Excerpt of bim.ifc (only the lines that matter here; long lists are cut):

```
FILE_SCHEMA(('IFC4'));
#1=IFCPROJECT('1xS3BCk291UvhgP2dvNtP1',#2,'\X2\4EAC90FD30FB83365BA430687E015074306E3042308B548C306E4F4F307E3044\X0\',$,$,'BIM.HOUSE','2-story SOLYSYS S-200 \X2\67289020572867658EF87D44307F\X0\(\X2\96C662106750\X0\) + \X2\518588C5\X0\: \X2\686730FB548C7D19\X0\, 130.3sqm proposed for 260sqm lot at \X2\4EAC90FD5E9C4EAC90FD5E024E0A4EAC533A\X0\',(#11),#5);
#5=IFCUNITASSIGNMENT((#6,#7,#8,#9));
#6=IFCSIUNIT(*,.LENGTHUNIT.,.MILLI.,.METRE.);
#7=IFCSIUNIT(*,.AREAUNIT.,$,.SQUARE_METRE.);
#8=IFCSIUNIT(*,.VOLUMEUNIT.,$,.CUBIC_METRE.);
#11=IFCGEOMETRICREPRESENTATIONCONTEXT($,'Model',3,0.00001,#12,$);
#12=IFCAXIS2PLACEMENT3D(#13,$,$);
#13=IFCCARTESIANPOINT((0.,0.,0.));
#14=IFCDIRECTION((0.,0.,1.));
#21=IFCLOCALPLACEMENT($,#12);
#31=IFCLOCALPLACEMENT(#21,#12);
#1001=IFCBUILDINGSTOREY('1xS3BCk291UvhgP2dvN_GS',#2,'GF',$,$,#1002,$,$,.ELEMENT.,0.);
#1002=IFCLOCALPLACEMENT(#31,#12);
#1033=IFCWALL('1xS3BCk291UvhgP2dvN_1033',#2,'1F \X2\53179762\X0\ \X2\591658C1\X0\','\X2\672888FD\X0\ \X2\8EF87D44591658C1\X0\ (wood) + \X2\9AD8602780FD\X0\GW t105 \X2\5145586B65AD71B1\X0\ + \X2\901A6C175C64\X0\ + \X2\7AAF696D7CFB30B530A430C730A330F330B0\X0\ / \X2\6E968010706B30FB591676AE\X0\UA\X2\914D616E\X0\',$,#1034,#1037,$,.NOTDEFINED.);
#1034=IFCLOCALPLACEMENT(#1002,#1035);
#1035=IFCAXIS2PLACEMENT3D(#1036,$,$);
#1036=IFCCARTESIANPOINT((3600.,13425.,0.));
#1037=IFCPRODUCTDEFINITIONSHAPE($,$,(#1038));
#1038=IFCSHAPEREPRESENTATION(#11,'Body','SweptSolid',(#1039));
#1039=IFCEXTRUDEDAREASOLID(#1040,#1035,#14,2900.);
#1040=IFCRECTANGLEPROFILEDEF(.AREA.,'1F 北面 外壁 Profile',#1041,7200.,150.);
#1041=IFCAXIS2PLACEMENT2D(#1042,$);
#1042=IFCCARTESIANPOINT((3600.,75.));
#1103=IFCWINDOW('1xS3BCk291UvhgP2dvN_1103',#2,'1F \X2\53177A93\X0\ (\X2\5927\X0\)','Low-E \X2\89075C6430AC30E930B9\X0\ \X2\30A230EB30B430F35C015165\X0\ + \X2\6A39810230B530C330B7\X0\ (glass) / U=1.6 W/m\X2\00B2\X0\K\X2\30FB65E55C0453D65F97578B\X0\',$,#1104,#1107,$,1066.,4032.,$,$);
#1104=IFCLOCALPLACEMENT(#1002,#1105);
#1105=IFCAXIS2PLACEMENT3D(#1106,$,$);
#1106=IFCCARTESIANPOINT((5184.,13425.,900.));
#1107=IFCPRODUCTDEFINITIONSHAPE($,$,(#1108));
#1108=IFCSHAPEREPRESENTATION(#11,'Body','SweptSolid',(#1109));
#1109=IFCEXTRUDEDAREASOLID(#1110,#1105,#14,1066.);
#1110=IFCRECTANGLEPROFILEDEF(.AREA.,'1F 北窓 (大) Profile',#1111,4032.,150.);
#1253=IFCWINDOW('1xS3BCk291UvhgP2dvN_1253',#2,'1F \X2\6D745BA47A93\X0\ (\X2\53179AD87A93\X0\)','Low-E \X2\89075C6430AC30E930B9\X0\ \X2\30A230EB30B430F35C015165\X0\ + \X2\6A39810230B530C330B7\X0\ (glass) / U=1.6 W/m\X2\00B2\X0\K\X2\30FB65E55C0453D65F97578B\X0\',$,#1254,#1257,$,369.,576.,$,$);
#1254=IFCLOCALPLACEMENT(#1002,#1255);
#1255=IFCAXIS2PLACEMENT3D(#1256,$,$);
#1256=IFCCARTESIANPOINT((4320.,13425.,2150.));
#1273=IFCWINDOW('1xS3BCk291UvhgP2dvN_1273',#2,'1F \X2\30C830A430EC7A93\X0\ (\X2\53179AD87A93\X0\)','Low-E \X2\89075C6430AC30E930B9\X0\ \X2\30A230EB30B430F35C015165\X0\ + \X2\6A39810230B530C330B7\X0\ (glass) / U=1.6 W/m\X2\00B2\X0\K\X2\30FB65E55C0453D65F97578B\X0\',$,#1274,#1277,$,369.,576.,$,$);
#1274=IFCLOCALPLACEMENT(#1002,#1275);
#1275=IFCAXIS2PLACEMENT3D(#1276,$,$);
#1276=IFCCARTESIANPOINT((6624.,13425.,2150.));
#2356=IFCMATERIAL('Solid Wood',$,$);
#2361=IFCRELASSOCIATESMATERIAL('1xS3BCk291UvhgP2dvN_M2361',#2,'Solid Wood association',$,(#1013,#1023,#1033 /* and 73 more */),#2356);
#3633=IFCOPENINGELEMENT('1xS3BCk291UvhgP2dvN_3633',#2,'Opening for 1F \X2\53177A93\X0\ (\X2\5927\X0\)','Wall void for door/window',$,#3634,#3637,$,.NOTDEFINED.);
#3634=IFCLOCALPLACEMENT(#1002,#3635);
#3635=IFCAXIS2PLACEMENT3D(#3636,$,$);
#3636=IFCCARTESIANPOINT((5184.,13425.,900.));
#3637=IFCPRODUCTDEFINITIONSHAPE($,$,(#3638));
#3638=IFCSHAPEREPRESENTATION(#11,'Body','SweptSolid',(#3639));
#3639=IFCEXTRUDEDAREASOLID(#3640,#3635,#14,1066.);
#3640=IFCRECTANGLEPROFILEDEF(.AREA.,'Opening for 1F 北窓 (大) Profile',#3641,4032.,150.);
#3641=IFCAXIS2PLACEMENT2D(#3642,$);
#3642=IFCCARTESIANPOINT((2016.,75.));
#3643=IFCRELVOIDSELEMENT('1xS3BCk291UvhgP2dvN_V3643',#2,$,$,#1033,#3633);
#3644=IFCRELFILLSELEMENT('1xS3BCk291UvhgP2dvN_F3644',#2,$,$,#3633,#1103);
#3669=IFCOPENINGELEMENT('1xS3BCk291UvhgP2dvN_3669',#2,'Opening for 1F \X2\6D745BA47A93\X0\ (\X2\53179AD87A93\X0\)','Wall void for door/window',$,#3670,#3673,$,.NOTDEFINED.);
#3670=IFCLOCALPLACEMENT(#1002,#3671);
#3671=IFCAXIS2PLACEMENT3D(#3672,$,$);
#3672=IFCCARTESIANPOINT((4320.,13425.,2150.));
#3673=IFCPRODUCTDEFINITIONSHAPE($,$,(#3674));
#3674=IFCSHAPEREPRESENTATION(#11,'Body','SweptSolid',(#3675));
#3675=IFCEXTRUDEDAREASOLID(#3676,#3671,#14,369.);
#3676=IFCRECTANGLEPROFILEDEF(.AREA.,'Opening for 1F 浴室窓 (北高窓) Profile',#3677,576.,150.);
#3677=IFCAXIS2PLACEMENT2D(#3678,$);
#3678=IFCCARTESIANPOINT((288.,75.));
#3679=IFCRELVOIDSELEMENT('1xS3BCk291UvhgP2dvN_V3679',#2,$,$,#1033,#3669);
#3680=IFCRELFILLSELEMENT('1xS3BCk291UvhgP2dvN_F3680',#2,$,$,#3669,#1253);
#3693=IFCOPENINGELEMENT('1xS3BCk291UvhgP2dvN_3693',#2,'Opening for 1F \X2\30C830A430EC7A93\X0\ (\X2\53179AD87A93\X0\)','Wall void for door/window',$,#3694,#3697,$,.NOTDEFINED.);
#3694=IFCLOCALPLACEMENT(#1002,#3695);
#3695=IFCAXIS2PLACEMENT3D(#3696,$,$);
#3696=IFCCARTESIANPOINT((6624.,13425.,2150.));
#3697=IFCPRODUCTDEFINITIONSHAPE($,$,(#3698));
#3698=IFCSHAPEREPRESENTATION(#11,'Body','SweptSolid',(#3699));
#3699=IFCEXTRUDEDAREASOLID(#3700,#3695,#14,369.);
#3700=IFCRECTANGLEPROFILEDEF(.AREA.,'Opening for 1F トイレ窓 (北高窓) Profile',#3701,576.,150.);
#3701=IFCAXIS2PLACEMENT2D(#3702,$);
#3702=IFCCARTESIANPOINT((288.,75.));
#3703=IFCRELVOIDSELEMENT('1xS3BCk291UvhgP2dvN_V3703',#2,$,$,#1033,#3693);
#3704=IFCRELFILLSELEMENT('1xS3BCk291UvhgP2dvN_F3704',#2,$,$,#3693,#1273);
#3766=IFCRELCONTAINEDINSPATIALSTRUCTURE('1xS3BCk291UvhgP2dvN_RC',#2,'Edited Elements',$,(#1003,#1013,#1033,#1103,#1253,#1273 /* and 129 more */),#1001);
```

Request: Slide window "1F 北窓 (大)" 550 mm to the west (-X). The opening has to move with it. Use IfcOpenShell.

```python
import ifcopenshell
import ifcopenshell.api.geometry
import ifcopenshell.util.placement
import ifcopenshell.util.unit

model = ifcopenshell.open("bim.ifc")
unit_scale = ifcopenshell.util.unit.calculate_unit_scale(model)

window = model.by_guid("1xS3BCk291UvhgP2dvN_1103")
opening = window.FillsVoids[0].RelatingOpeningElement
wall = opening.VoidsElements[0].RelatingBuildingElement

wall_matrix = ifcopenshell.util.placement.get_local_placement(wall.ObjectPlacement)
shift = wall_matrix[:3, 0] * -0.55 / unit_scale
before = ifcopenshell.util.placement.get_local_placement(window.ObjectPlacement)[:3, 3].copy()

# The window is not placed relative to its opening, so move both.
for product in (opening, window):
    matrix = ifcopenshell.util.placement.get_local_placement(product.ObjectPlacement)
    matrix[:3, 3] += shift
    ifcopenshell.api.geometry.edit_object_placement(model, product=product, matrix=matrix, is_si=False)

after = ifcopenshell.util.placement.get_local_placement(window.ObjectPlacement)[:3, 3]
print("window moved by", (after - before).round(3) + 0.0)

model.write("bim_v2.ifc")
```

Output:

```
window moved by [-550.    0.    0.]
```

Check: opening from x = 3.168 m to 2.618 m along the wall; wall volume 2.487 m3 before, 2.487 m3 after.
